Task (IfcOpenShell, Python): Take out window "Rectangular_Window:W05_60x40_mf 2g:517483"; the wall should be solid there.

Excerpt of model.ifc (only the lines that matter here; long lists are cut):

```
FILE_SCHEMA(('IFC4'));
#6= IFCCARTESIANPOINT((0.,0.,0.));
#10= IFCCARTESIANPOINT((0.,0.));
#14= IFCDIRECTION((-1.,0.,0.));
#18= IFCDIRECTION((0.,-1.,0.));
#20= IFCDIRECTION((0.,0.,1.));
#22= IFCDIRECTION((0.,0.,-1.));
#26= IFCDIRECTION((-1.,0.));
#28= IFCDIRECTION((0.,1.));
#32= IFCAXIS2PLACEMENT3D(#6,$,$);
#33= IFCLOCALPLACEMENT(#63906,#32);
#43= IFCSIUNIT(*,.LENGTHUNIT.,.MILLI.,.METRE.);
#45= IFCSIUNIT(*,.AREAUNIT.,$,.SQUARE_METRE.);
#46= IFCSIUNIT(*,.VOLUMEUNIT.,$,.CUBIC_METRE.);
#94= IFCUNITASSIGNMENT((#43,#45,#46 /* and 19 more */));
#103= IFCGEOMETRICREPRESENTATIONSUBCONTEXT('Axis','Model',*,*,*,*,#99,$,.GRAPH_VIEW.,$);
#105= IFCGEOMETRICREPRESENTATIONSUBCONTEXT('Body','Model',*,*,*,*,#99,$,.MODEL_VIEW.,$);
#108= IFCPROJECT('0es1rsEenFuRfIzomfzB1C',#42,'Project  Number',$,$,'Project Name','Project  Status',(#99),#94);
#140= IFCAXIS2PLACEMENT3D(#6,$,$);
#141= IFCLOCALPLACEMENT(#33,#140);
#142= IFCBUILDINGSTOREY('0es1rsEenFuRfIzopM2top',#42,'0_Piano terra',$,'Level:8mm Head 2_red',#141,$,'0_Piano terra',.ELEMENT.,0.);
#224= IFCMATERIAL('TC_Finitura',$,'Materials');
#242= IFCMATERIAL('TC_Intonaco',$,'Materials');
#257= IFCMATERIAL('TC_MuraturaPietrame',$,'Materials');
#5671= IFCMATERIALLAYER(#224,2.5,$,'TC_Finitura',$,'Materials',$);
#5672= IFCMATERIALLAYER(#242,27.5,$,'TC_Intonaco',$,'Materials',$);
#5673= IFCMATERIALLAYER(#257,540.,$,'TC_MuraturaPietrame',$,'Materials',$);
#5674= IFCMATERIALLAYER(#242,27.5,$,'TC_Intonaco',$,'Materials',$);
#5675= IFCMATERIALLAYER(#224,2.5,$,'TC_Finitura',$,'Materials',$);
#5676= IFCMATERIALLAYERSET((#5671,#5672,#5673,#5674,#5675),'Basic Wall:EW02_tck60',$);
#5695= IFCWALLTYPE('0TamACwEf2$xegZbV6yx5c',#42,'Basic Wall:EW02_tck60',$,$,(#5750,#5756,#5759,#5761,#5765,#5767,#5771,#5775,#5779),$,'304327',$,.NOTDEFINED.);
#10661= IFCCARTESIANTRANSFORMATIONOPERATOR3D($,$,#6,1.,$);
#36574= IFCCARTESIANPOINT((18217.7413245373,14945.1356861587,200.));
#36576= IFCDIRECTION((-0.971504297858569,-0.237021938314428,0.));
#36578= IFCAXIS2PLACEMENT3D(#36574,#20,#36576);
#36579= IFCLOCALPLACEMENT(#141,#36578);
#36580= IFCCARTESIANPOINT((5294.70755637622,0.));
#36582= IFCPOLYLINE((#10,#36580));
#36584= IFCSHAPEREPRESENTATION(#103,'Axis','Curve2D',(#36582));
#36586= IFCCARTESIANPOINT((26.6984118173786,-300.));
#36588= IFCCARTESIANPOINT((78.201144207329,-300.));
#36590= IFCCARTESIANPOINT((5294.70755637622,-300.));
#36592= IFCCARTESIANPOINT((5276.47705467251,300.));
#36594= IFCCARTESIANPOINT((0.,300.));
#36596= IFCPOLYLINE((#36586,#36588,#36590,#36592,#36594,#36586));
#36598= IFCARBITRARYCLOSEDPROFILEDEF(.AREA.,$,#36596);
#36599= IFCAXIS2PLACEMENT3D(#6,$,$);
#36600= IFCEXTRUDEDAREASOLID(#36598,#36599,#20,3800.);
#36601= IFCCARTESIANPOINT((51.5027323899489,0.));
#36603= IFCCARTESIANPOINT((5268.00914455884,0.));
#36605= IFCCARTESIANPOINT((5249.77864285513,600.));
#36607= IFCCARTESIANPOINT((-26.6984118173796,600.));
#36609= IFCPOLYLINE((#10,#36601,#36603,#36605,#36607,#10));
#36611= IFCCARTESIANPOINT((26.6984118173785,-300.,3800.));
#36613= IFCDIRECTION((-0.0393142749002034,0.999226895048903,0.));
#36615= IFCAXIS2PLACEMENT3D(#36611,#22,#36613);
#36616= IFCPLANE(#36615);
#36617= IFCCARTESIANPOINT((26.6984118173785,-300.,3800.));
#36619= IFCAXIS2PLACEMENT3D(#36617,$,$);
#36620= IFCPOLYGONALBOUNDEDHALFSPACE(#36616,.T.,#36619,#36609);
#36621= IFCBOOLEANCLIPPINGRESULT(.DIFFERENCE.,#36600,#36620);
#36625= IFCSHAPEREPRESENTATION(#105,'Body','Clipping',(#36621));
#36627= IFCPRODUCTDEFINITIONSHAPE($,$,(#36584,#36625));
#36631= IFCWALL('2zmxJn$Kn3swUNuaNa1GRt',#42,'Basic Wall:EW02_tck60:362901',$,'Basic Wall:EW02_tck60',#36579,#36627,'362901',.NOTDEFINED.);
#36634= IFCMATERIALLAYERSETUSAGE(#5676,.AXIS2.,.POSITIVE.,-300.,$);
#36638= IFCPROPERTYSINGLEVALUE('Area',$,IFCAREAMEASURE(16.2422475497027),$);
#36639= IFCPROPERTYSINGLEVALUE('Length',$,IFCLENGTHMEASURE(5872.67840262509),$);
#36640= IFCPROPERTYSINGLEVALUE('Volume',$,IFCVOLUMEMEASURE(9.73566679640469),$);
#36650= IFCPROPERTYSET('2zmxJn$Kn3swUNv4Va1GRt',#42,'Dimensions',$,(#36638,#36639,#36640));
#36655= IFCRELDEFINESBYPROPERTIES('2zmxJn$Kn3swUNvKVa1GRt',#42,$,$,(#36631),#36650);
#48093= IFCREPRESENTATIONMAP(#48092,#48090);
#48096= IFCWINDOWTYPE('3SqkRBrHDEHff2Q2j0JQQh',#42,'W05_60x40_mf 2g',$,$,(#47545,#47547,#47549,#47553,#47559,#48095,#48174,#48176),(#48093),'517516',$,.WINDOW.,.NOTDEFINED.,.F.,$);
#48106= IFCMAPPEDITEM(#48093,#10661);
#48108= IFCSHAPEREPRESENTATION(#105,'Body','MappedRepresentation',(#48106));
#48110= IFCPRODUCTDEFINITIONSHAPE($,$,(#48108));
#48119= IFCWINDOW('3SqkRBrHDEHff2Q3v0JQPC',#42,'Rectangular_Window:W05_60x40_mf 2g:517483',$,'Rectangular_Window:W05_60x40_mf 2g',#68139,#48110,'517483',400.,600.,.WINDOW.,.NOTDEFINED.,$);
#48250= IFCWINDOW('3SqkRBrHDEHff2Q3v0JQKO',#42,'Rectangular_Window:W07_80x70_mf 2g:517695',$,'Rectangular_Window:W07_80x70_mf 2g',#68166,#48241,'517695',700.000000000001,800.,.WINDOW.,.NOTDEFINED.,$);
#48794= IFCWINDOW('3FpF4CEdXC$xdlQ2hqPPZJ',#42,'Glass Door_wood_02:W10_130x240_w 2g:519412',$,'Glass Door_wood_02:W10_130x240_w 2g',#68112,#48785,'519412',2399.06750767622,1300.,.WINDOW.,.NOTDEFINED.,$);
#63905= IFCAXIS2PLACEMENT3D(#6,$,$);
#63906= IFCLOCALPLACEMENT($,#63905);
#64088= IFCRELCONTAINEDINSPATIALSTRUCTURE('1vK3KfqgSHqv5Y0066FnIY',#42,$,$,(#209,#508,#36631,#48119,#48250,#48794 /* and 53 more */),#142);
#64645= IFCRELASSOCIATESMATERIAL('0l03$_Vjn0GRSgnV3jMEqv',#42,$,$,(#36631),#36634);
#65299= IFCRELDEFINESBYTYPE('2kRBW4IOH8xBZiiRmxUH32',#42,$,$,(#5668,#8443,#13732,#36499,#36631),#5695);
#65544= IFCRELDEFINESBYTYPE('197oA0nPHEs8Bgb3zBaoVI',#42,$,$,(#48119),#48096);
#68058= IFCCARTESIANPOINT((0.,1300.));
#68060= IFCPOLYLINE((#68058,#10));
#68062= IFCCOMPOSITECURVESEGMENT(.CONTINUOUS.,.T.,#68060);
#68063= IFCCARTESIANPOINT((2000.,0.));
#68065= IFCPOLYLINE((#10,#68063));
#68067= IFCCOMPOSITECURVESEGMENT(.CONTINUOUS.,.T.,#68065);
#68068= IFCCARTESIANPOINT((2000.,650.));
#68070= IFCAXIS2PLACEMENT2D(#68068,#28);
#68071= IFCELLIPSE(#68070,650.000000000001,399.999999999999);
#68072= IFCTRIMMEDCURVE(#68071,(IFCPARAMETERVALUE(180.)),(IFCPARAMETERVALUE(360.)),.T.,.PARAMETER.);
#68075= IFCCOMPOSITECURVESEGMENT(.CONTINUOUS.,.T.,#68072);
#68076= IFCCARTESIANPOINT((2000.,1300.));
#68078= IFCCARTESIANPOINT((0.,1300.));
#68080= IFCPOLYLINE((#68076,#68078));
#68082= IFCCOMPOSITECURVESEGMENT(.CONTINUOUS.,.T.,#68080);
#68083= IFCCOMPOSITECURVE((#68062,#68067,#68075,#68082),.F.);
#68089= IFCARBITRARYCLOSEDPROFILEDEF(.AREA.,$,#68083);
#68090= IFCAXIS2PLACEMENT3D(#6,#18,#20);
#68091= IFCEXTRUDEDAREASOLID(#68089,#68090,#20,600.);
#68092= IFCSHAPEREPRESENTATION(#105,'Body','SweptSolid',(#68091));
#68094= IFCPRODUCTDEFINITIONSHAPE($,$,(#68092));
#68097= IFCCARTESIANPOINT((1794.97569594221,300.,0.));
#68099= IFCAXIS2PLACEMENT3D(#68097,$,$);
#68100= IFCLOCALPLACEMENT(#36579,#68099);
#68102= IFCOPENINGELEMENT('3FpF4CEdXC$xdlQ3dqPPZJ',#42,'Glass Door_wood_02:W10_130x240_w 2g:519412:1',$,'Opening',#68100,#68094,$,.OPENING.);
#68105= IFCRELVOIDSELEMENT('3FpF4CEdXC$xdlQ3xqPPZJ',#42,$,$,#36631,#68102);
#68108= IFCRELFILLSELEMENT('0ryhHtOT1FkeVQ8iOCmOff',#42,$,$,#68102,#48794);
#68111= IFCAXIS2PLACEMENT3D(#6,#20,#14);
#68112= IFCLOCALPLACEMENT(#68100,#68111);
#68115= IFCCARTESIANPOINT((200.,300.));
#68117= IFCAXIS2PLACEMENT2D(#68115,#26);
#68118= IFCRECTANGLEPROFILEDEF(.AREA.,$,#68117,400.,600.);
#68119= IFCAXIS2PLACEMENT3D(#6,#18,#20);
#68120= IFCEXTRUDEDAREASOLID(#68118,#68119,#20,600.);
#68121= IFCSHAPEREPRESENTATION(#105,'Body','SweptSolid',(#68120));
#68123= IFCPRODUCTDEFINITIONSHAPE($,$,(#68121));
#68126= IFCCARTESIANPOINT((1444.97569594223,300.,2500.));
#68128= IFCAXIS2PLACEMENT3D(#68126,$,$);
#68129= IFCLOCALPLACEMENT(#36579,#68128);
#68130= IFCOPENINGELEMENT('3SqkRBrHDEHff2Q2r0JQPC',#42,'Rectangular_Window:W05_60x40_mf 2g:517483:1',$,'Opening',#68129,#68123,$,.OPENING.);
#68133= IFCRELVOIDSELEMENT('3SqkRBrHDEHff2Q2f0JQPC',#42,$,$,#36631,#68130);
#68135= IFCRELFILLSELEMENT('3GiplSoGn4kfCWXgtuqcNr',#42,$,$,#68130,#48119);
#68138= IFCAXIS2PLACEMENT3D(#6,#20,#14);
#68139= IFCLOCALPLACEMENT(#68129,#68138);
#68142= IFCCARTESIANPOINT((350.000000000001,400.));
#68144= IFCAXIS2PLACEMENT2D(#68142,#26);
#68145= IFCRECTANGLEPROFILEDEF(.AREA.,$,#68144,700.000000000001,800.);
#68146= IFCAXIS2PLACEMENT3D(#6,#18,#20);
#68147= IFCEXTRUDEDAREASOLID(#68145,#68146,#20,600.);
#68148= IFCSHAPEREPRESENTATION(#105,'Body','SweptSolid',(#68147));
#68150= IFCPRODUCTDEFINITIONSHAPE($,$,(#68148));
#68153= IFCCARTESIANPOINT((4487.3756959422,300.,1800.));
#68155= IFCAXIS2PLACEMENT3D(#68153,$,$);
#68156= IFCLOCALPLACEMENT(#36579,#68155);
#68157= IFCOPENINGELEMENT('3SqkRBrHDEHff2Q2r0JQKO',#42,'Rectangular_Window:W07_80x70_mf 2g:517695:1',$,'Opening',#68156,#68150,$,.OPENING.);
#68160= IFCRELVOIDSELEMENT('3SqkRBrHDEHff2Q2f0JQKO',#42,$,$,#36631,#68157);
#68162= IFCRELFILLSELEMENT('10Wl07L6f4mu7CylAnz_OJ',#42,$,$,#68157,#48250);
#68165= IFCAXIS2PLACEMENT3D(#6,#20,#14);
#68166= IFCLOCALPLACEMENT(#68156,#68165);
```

```python
import ifcopenshell
import ifcopenshell.api.feature
import ifcopenshell.api.pset
import ifcopenshell.api.root
import ifcopenshell.geom
import ifcopenshell.util.element
import ifcopenshell.util.shape
import ifcopenshell.util.unit

model = ifcopenshell.open("model.ifc")
area_scale = ifcopenshell.util.unit.calculate_unit_scale(model, "AREAUNIT")
volume_scale = ifcopenshell.util.unit.calculate_unit_scale(model, "VOLUMEUNIT")
settings = ifcopenshell.geom.settings()


def volume(element):
    """Net volume in cubic metres, openings subtracted."""
    shape = ifcopenshell.geom.create_shape(settings, element)
    return ifcopenshell.util.shape.get_volume(shape.geometry)


window = model.by_id(48119)
opening = window.FillsVoids[0].RelatingOpeningElement
wall = opening.VoidsElements[0].RelatingBuildingElement
before = volume(wall)

ifcopenshell.api.root.remove_product(model, product=window)
ifcopenshell.api.feature.remove_feature(model, feature=opening)

after = volume(wall)
thickness = 0.6  # wall thickness in metres

# Update the wall's stored quantities.
pset = model.by_id(ifcopenshell.util.element.get_pset(wall, "Dimensions", should_inherit=False)["id"])
ifcopenshell.api.pset.edit_pset(model, pset=pset, properties={
    "Area": model.create_entity("IfcAreaMeasure", after / thickness / area_scale),
    "Volume": model.create_entity("IfcVolumeMeasure", after / volume_scale),
})

print(f"wall volume {before:.3f} -> {after:.3f} m3")

model.write("model_rev.ifc")
```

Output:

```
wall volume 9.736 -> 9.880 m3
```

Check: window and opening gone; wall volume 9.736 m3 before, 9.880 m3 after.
